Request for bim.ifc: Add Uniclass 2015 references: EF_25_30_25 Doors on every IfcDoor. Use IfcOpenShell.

First a look at what the model holds.

```python
import ifcopenshell

model = ifcopenshell.open("bim.ifc")
print(model.schema)
print("classifications:", [c.Name for c in model.by_type("IfcClassification")])
for ifc_class in ("IfcDoor", "IfcRoof", "IfcStair", "IfcWall", "IfcWindow"):
    print(ifc_class, len(model.by_type(ifc_class)))
```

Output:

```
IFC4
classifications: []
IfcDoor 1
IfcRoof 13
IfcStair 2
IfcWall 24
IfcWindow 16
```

```python
import ifcopenshell
import ifcopenshell.api.classification

model = ifcopenshell.open("bim.ifc")

system = ifcopenshell.api.classification.add_classification(model, classification="Uniclass 2015")

codes = {
    "IfcDoor": ("EF_25_30_25", "Doors"),
}
for ifc_class, (code, name) in codes.items():
    products = model.by_type(ifc_class)
    ifcopenshell.api.classification.add_reference(
        model, products=products, classification=system, identification=code, name=name
    )
    print(code, len(products))

model.write("bim_v2.ifc")
```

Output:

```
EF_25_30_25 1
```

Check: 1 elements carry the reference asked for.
